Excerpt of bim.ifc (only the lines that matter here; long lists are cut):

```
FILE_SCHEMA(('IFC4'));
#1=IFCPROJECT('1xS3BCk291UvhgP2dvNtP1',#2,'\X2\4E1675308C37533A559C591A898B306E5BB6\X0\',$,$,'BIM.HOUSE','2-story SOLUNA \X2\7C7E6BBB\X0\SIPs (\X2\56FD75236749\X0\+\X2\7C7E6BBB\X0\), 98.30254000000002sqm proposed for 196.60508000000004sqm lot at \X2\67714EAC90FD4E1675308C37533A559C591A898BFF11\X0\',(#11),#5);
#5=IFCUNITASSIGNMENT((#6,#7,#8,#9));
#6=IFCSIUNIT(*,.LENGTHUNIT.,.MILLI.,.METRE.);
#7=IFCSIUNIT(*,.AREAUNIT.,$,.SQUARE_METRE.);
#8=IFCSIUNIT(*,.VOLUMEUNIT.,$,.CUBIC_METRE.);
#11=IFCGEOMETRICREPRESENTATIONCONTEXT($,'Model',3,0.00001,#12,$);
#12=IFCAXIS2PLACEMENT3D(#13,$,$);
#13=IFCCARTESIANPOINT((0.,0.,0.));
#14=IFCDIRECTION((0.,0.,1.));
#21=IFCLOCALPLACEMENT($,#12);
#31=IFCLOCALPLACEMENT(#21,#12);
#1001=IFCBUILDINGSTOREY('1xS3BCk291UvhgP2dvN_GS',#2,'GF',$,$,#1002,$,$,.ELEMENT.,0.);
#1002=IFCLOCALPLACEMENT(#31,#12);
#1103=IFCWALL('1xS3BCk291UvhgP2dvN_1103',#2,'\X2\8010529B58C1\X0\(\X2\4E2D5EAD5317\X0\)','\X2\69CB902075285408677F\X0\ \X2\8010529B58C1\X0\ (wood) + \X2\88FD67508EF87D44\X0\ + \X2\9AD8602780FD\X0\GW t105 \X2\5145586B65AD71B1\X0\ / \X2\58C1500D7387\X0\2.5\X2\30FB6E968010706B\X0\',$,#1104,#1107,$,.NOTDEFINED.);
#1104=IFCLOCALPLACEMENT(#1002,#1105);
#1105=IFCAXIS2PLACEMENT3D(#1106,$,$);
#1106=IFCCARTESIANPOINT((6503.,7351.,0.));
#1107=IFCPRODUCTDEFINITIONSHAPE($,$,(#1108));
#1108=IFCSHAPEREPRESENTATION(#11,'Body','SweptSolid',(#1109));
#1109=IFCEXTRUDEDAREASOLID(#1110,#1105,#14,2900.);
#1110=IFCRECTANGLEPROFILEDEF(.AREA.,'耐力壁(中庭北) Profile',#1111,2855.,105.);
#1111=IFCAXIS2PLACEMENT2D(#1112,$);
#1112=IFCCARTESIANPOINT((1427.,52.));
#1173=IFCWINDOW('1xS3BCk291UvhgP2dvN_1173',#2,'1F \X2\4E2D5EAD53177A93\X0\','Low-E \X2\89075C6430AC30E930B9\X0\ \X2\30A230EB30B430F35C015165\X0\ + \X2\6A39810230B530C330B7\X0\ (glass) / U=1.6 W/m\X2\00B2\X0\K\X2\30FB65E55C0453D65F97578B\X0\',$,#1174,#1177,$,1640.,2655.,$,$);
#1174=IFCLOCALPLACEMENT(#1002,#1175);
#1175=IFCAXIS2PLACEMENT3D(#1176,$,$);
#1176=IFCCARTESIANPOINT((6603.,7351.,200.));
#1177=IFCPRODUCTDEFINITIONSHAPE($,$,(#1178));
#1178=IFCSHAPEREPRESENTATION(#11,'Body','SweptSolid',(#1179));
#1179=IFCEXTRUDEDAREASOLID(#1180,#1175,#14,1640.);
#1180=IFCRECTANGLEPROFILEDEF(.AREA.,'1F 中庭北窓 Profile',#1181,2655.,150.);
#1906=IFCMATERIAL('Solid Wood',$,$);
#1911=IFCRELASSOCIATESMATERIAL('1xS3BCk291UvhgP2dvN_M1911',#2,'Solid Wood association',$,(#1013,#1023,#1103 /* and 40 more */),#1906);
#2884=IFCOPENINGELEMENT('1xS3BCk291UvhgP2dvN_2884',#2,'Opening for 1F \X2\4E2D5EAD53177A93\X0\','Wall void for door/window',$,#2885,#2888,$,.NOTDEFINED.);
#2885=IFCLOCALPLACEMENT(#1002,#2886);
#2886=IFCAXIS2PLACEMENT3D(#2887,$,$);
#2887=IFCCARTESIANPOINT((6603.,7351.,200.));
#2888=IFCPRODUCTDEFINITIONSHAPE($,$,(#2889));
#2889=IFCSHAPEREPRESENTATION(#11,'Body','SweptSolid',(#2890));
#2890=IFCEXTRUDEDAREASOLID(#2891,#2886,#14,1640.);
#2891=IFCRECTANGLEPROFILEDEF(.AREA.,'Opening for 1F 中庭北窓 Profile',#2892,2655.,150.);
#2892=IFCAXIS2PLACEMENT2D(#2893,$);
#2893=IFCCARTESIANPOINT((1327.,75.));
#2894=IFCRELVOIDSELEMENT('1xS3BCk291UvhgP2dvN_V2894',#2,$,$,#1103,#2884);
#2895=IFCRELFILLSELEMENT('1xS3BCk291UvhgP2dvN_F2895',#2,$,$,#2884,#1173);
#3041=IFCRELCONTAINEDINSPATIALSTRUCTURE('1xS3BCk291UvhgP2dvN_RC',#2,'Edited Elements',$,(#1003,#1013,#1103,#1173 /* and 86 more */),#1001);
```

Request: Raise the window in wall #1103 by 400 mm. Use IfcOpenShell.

```python
import numpy as np
import ifcopenshell
import ifcopenshell.api.geometry
import ifcopenshell.util.placement
import ifcopenshell.util.unit

model = ifcopenshell.open("bim.ifc")
unit_scale = ifcopenshell.util.unit.calculate_unit_scale(model)

window = model.by_id(1173)
opening = window.FillsVoids[0].RelatingOpeningElement
dz = 400.0

shift = np.array([0.0, 0.0, dz])
# The window is not placed relative to its opening, so move both.
for product in (opening, window):
    matrix = ifcopenshell.util.placement.get_local_placement(product.ObjectPlacement)
    matrix[:3, 3] += shift
    ifcopenshell.api.geometry.edit_object_placement(model, product=product, matrix=matrix, is_si=False)

print(f"moved by {dz * unit_scale:+.3f} m")

model.write("bim_v2.ifc")
```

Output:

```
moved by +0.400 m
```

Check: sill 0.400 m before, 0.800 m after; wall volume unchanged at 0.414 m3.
